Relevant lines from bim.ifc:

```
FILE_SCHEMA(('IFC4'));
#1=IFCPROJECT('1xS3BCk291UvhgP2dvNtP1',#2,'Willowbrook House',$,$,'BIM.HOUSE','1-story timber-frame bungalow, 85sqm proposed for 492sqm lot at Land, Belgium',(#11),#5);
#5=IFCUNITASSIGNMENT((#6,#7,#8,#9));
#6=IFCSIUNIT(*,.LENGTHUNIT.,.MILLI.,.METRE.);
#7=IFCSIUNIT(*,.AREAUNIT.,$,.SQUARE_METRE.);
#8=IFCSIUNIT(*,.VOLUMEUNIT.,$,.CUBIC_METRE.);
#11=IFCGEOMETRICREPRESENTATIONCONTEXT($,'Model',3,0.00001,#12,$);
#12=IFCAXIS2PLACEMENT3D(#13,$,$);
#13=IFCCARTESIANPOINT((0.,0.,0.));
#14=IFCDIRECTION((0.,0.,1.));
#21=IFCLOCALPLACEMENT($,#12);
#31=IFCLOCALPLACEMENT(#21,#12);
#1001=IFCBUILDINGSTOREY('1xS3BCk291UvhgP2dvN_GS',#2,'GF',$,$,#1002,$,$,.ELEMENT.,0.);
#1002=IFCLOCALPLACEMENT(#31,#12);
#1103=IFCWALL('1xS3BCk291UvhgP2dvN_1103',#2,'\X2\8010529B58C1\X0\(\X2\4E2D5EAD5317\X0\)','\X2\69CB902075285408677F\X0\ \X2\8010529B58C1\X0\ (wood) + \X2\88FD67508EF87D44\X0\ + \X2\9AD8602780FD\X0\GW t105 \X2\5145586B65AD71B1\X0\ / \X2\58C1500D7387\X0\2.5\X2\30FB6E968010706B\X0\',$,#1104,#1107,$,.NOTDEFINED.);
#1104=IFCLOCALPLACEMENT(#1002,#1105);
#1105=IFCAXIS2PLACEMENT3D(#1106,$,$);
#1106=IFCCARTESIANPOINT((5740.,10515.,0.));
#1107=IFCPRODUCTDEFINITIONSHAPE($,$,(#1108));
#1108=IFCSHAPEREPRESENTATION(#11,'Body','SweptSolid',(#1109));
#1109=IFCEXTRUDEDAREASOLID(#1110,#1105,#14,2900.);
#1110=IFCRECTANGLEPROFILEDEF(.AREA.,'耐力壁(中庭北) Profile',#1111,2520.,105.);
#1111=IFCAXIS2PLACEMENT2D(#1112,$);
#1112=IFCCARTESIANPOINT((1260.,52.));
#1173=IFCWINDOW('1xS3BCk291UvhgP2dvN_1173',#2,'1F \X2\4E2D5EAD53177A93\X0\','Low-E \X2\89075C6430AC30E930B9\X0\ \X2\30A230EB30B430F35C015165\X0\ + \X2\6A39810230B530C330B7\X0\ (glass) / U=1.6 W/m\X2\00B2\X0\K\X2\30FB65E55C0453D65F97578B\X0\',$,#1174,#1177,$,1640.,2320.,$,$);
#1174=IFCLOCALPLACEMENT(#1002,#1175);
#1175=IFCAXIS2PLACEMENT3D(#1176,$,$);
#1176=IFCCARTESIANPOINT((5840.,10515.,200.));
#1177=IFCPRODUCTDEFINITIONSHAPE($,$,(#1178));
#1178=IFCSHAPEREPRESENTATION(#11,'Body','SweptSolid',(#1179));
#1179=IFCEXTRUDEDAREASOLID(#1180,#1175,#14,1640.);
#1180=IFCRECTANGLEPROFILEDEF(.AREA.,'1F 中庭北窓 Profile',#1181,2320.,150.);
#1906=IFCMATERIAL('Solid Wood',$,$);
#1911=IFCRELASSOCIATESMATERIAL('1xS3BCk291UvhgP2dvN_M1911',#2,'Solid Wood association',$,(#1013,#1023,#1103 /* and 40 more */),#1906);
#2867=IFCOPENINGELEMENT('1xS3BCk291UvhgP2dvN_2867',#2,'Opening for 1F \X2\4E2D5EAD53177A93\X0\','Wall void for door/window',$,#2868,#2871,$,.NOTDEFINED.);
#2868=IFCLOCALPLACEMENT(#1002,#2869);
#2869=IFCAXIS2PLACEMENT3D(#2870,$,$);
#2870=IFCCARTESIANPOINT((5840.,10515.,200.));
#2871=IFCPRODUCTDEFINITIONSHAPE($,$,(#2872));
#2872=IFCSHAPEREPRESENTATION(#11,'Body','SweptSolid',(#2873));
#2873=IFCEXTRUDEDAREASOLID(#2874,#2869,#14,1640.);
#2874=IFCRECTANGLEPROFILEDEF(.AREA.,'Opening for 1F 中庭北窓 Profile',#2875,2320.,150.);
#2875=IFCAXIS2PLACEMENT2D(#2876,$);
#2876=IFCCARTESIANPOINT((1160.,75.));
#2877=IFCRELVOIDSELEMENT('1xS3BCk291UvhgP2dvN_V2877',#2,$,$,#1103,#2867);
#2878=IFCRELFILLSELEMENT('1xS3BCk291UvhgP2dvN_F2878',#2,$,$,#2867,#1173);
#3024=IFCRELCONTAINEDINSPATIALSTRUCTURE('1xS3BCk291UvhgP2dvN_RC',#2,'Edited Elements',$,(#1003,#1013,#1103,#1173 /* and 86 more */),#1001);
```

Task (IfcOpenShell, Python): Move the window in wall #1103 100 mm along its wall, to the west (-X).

```python
import ifcopenshell
import ifcopenshell.api.geometry
import ifcopenshell.util.placement
import ifcopenshell.util.unit

model = ifcopenshell.open("bim.ifc")
unit_scale = ifcopenshell.util.unit.calculate_unit_scale(model)

window = model.by_guid("1xS3BCk291UvhgP2dvN_1173")
opening = window.FillsVoids[0].RelatingOpeningElement
wall = opening.VoidsElements[0].RelatingBuildingElement

wall_matrix = ifcopenshell.util.placement.get_local_placement(wall.ObjectPlacement)
shift = wall_matrix[:3, 0] * -0.1 / unit_scale
before = ifcopenshell.util.placement.get_local_placement(window.ObjectPlacement)[:3, 3].copy()

# The window is not placed relative to its opening, so move both.
for product in (opening, window):
    matrix = ifcopenshell.util.placement.get_local_placement(product.ObjectPlacement)
    matrix[:3, 3] += shift
    ifcopenshell.api.geometry.edit_object_placement(model, product=product, matrix=matrix, is_si=False)

after = ifcopenshell.util.placement.get_local_placement(window.ObjectPlacement)[:3, 3]
print("window moved by", (after - before).round(3) + 0.0)

model.write("bim-out.ifc")
```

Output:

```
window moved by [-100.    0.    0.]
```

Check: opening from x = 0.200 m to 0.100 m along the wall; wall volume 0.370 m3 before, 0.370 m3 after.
